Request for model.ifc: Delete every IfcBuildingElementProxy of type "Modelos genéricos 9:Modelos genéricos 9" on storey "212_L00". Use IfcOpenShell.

First a look at what the model holds.

```python
import ifcopenshell
import ifcopenshell.util.element

model = ifcopenshell.open("model.ifc")
print(model.schema)
storey = next(s for s in model.by_type("IfcBuildingStorey") if s.Name == "212_L00")
proxies = [e for e in ifcopenshell.util.element.get_decomposition(storey) if e.is_a("IfcBuildingElementProxy")]
seen = {}
for e in proxies:
    element_type = ifcopenshell.util.element.get_type(e)
    name = element_type.Name if element_type not in (None, e) else None
    seen[name] = seen.get(name, 0) + 1
for name, count in sorted(seen.items(), key=str):
    print(count, "x", name)
```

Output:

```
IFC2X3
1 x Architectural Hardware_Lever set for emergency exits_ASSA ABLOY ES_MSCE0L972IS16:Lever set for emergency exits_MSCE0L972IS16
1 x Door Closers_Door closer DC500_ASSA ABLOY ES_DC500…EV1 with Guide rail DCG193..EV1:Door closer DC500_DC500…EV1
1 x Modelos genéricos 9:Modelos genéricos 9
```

```python
import ifcopenshell
import ifcopenshell.api.root
import ifcopenshell.util.element

model = ifcopenshell.open("model.ifc")

storey = next(s for s in model.by_type("IfcBuildingStorey") if s.Name == "212_L00")
proxies = [e for e in ifcopenshell.util.element.get_decomposition(storey) if e.is_a("IfcBuildingElementProxy")]
targets = [e for e in proxies if (t := ifcopenshell.util.element.get_type(e)) not in (None, e) and t.Name == "Modelos genéricos 9:Modelos genéricos 9"]

for e in targets:
    ifcopenshell.api.root.remove_product(model, product=e)
print(len(targets), "removed")

model.write("model-out.ifc")
```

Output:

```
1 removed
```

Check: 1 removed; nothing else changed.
